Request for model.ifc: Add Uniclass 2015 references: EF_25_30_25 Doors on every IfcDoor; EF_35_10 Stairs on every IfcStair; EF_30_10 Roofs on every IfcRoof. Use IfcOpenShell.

First a look at what the model holds.

```python
import ifcopenshell

model = ifcopenshell.open("model.ifc")
print(model.schema)
print("classifications:", [c.Name for c in model.by_type("IfcClassification")])
for ifc_class in ("IfcDoor", "IfcRoof", "IfcStair", "IfcWall", "IfcWindow"):
    print(ifc_class, len(model.by_type(ifc_class)))
```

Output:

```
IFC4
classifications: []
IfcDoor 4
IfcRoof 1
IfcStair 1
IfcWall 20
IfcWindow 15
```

```python
import ifcopenshell
import ifcopenshell.api.classification

model = ifcopenshell.open("model.ifc")

system = ifcopenshell.api.classification.add_classification(model, classification="Uniclass 2015")

codes = {
    "IfcDoor": ("EF_25_30_25", "Doors"),
    "IfcStair": ("EF_35_10", "Stairs"),
    "IfcRoof": ("EF_30_10", "Roofs"),
}
for ifc_class, (code, name) in codes.items():
    products = model.by_type(ifc_class)
    ifcopenshell.api.classification.add_reference(
        model, products=products, classification=system, identification=code, name=name
    )
    print(code, len(products))

model.write("model_updated.ifc")
```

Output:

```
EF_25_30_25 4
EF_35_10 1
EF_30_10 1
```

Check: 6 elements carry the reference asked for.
